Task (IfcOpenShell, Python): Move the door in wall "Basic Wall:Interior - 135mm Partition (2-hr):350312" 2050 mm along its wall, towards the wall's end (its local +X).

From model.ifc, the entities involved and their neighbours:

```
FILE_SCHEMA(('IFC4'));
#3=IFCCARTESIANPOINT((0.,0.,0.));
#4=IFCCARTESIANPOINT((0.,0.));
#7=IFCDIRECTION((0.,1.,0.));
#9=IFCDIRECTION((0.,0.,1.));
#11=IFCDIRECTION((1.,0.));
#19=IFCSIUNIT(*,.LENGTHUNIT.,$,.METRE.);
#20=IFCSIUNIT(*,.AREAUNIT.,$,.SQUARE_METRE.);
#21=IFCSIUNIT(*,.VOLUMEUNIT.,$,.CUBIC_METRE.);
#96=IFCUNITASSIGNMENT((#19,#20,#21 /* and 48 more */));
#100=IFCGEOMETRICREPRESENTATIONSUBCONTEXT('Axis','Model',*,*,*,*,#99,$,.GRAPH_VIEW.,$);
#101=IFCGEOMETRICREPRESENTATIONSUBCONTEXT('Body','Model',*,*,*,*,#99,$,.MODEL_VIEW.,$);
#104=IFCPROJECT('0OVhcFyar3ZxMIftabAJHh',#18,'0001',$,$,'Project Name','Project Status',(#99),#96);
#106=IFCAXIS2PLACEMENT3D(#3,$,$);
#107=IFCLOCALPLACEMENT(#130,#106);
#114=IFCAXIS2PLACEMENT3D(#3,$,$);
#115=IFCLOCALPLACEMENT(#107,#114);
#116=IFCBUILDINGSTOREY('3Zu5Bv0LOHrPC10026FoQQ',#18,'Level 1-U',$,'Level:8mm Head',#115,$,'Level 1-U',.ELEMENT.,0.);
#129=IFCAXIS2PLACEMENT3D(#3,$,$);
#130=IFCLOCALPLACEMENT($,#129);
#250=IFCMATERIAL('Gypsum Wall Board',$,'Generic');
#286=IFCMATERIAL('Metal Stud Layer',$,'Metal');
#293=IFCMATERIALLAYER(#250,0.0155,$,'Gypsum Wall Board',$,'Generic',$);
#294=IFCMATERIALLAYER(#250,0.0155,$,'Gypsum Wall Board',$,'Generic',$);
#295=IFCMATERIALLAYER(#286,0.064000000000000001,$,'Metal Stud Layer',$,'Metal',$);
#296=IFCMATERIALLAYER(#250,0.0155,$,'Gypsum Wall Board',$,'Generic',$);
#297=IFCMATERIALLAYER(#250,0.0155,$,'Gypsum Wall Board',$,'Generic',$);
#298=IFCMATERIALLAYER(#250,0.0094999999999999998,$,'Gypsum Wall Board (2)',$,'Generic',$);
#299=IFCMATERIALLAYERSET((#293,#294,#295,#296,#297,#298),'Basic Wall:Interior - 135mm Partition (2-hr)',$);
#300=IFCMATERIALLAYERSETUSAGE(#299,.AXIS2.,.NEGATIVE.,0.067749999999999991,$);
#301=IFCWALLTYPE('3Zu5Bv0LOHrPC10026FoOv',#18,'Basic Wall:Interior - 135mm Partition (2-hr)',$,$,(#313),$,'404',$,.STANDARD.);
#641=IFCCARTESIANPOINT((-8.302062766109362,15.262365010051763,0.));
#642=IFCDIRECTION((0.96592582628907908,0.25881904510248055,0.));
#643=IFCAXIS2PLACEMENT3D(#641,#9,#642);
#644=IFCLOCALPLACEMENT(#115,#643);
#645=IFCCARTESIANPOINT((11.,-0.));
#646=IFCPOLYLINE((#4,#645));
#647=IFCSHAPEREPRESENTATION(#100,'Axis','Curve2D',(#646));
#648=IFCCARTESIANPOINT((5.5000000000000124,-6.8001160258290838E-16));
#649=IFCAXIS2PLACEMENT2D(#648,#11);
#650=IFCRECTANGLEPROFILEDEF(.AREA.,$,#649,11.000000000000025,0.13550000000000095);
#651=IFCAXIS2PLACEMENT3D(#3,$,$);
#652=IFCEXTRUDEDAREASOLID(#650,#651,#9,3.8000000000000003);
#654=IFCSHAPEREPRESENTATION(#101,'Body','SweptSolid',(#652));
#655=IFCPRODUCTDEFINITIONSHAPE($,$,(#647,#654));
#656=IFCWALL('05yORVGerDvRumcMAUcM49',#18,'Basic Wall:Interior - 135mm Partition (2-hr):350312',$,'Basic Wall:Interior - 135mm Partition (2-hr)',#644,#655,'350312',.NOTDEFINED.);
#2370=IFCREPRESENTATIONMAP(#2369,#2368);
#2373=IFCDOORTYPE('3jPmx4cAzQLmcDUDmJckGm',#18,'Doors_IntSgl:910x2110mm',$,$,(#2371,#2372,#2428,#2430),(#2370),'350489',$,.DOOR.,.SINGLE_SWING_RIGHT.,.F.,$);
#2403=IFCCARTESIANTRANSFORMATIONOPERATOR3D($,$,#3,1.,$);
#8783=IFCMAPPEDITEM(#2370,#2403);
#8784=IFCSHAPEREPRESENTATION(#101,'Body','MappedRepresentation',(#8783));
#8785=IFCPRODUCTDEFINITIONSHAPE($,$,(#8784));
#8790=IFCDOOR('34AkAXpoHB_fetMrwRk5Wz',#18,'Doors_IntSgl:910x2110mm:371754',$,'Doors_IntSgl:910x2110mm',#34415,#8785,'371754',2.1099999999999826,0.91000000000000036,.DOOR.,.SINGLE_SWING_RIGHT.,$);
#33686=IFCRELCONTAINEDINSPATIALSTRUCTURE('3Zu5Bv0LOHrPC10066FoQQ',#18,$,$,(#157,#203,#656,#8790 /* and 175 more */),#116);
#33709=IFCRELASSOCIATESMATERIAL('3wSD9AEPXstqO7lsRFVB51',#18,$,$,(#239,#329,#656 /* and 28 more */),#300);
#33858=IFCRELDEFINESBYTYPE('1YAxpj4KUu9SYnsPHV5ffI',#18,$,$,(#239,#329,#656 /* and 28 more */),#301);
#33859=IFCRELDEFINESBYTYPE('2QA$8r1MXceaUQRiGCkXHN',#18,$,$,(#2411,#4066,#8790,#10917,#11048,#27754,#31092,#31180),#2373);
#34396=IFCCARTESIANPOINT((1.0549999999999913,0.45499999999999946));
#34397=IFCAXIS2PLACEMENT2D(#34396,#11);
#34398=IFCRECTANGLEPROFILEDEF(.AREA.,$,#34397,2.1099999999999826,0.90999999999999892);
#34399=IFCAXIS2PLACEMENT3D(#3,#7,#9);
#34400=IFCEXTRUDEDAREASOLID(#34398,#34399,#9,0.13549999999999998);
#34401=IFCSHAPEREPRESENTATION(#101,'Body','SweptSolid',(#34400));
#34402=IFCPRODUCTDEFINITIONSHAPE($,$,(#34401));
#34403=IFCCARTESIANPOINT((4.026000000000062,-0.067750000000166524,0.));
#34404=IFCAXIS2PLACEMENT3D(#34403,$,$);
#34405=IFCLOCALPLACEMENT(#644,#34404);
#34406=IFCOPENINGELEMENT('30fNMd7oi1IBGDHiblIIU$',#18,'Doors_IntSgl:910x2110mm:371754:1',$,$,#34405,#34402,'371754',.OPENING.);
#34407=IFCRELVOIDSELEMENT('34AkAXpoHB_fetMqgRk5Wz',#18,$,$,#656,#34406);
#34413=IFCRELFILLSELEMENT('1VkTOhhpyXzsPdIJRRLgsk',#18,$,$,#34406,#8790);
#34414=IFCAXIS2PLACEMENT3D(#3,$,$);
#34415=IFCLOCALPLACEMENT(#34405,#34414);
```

```python
import ifcopenshell
import ifcopenshell.api.geometry
import ifcopenshell.util.placement

model = ifcopenshell.open("model.ifc")

door = model.by_guid("34AkAXpoHB_fetMrwRk5Wz")
opening = door.FillsVoids[0].RelatingOpeningElement
wall = opening.VoidsElements[0].RelatingBuildingElement

wall_matrix = ifcopenshell.util.placement.get_local_placement(wall.ObjectPlacement)
shift = wall_matrix[:3, 0] * 2.05
before = ifcopenshell.util.placement.get_local_placement(door.ObjectPlacement)[:3, 3].copy()

# The door is placed relative to its opening, so it follows when the opening moves.
matrix = ifcopenshell.util.placement.get_local_placement(opening.ObjectPlacement)
matrix[:3, 3] += shift
ifcopenshell.api.geometry.edit_object_placement(
    model, product=opening, matrix=matrix, is_si=False, should_transform_children=True
)

after = ifcopenshell.util.placement.get_local_placement(door.ObjectPlacement)[:3, 3]
print("door moved by", (after - before).round(3) + 0.0)

model.write("model-out.ifc")
```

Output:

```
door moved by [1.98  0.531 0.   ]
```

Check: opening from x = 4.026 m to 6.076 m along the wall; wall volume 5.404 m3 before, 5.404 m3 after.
